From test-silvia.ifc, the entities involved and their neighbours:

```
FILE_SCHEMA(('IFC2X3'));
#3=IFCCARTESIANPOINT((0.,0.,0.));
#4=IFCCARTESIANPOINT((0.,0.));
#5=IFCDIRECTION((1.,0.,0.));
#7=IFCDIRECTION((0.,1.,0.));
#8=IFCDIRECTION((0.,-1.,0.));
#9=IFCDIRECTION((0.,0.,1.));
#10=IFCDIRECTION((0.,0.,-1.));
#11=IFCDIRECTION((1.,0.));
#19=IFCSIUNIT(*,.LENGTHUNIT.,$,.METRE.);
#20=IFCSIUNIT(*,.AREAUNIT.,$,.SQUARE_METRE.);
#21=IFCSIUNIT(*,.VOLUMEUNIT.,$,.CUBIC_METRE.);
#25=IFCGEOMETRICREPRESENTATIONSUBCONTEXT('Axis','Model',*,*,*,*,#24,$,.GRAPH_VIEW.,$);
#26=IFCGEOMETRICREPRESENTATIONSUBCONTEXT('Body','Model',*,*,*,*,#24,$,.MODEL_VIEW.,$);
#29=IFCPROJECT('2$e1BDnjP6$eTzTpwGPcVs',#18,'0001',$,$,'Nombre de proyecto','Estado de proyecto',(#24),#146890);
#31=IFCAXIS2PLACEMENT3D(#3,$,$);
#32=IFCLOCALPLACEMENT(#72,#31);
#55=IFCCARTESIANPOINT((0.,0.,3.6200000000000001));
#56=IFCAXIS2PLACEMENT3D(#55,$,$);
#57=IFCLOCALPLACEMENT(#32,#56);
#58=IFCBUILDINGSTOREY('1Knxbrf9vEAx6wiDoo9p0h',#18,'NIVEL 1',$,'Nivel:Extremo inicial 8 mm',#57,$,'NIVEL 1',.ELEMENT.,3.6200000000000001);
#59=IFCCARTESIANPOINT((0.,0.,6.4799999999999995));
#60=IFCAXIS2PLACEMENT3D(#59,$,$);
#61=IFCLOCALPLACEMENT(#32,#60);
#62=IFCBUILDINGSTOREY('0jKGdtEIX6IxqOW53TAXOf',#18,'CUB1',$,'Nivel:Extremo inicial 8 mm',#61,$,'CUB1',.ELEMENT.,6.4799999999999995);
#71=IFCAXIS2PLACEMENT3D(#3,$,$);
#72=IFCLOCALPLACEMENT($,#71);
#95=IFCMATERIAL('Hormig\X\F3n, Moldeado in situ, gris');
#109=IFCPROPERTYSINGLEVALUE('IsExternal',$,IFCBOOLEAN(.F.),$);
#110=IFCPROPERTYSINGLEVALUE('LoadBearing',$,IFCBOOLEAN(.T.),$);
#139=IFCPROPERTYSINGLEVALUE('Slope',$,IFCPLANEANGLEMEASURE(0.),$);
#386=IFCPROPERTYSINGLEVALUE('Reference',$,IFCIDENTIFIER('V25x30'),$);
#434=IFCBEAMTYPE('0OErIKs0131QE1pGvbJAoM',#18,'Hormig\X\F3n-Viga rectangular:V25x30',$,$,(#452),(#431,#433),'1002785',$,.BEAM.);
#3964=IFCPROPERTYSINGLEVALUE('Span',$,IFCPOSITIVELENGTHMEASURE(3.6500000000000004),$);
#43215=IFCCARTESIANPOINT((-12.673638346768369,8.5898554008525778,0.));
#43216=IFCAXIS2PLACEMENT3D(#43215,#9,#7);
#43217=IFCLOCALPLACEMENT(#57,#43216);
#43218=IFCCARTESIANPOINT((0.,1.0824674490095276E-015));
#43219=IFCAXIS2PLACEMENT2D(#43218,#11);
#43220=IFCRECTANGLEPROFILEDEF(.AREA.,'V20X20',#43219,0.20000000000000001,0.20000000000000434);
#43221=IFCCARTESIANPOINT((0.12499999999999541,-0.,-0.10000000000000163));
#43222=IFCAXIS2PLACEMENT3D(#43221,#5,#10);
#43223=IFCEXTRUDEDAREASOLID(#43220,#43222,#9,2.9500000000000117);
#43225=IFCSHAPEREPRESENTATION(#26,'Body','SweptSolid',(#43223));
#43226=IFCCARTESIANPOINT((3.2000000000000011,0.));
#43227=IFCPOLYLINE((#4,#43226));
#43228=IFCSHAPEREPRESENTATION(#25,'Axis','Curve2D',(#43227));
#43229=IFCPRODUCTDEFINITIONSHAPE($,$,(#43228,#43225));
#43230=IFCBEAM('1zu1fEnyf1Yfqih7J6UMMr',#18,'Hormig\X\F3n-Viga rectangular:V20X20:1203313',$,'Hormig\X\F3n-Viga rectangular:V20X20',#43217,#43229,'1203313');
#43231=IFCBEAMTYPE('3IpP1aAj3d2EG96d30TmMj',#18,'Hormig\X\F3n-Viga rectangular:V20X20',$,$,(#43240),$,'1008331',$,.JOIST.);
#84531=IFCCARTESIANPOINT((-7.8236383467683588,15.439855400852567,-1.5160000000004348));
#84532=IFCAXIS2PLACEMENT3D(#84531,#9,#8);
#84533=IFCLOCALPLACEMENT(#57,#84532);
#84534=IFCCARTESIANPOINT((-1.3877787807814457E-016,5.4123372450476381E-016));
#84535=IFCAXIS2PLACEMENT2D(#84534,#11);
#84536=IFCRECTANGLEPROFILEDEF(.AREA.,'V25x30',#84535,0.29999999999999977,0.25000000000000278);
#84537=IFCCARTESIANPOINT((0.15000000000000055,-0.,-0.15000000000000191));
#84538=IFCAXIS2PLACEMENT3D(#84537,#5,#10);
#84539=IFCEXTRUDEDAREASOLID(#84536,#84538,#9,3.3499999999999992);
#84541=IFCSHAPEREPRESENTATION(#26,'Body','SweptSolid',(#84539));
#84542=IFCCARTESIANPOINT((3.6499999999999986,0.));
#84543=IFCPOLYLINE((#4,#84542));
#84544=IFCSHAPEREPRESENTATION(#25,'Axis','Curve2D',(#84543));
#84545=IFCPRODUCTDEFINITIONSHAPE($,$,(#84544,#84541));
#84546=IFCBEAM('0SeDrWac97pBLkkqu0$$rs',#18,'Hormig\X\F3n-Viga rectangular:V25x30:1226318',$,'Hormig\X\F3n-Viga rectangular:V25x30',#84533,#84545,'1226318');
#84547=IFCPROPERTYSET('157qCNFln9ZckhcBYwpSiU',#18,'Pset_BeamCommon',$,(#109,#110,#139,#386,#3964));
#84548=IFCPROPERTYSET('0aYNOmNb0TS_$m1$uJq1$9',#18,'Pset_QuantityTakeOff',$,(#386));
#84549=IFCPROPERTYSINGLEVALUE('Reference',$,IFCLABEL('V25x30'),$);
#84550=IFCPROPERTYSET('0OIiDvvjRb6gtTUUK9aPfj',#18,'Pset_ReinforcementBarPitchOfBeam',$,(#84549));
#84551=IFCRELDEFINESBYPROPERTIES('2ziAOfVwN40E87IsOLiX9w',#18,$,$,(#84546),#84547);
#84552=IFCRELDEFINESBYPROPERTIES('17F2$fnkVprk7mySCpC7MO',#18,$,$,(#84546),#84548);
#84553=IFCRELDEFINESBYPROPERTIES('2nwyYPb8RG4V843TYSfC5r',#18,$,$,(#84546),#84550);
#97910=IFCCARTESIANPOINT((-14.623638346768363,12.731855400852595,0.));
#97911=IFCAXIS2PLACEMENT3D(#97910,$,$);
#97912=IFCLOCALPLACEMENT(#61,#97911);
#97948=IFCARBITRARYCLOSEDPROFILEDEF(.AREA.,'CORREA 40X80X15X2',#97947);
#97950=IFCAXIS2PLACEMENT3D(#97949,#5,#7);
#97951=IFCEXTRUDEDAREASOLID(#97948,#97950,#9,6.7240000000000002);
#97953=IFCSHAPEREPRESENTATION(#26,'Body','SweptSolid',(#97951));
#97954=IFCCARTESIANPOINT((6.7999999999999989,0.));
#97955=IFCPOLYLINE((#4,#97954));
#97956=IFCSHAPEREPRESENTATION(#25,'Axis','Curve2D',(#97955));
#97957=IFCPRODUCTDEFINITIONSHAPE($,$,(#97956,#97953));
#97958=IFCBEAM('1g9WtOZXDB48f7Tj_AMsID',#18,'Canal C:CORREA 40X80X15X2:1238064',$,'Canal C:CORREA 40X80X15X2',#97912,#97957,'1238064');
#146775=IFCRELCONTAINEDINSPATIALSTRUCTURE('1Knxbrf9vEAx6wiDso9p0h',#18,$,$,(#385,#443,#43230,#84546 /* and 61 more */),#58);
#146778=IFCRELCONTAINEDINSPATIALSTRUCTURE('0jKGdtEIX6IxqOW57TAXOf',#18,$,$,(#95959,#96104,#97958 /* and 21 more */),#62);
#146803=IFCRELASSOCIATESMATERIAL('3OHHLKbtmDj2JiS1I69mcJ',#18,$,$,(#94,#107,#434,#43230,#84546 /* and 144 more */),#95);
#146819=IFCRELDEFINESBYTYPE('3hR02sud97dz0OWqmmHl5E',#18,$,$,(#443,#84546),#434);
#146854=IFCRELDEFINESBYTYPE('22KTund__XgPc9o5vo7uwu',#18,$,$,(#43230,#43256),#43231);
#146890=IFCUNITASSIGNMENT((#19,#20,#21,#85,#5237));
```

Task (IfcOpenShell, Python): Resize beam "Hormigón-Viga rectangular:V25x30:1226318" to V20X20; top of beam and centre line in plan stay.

```python
import ifcopenshell
import ifcopenshell.api.pset
import ifcopenshell.api.type
import ifcopenshell.util.element
import ifcopenshell.util.representation

model = ifcopenshell.open("test-silvia.ifc")

member = model.by_id(84546)
source = next(p for p in model.by_type("IfcRectangleProfileDef") if p.ProfileName == "V20X20")

body = ifcopenshell.util.representation.get_representation(member, "Model", "Body")
solid = body.Items[0]
old_profile = solid.SweptArea

# Copy the section's sizes but keep this member's own profile position.
profile = ifcopenshell.util.element.copy(model, source)
# Profiles are centred, so shift by half the change in depth to hold the top.
shift = (old_profile.XDim - profile.XDim) / 2
x, y = old_profile.Position.Location.Coordinates
up = (-1.0, 0.0)  # upwards, in the solid's own plane
location = model.createIfcCartesianPoint((x + up[0] * shift, y + up[1] * shift))
profile.Position = model.createIfcAxis2Placement2D(location, old_profile.Position.RefDirection)
solid.SweptArea = profile
if not model.get_total_inverses(old_profile):
    ifcopenshell.util.element.remove_deep2(model, old_profile)

new_type = model.by_guid("3IpP1aAj3d2EG96d30TmMj")
ifcopenshell.api.type.assign_type(
    model, related_objects=[member], relating_type=new_type, should_map_representations=False
)
member.Name = member.Name.replace("V25x30", "V20X20")
member.ObjectType = "Hormigón-Viga rectangular:V20X20"
pset = model.by_id(ifcopenshell.util.element.get_pset(member, "Pset_BeamCommon", should_inherit=False)["id"])
ifcopenshell.api.pset.edit_pset(model, pset=pset, properties={"Reference": "V20X20"})
pset = model.by_id(ifcopenshell.util.element.get_pset(member, "Pset_QuantityTakeOff", should_inherit=False)["id"])
ifcopenshell.api.pset.edit_pset(model, pset=pset, properties={"Reference": "V20X20"})
pset = model.by_id(ifcopenshell.util.element.get_pset(member, "Pset_ReinforcementBarPitchOfBeam", should_inherit=False)["id"])
ifcopenshell.api.pset.edit_pset(model, pset=pset, properties={"Reference": "V20X20"})

print(solid.SweptArea)

model.write("test-silvia_edited.ifc")
```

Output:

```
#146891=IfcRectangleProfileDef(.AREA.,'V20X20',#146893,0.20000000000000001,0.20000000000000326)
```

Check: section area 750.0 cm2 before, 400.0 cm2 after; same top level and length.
